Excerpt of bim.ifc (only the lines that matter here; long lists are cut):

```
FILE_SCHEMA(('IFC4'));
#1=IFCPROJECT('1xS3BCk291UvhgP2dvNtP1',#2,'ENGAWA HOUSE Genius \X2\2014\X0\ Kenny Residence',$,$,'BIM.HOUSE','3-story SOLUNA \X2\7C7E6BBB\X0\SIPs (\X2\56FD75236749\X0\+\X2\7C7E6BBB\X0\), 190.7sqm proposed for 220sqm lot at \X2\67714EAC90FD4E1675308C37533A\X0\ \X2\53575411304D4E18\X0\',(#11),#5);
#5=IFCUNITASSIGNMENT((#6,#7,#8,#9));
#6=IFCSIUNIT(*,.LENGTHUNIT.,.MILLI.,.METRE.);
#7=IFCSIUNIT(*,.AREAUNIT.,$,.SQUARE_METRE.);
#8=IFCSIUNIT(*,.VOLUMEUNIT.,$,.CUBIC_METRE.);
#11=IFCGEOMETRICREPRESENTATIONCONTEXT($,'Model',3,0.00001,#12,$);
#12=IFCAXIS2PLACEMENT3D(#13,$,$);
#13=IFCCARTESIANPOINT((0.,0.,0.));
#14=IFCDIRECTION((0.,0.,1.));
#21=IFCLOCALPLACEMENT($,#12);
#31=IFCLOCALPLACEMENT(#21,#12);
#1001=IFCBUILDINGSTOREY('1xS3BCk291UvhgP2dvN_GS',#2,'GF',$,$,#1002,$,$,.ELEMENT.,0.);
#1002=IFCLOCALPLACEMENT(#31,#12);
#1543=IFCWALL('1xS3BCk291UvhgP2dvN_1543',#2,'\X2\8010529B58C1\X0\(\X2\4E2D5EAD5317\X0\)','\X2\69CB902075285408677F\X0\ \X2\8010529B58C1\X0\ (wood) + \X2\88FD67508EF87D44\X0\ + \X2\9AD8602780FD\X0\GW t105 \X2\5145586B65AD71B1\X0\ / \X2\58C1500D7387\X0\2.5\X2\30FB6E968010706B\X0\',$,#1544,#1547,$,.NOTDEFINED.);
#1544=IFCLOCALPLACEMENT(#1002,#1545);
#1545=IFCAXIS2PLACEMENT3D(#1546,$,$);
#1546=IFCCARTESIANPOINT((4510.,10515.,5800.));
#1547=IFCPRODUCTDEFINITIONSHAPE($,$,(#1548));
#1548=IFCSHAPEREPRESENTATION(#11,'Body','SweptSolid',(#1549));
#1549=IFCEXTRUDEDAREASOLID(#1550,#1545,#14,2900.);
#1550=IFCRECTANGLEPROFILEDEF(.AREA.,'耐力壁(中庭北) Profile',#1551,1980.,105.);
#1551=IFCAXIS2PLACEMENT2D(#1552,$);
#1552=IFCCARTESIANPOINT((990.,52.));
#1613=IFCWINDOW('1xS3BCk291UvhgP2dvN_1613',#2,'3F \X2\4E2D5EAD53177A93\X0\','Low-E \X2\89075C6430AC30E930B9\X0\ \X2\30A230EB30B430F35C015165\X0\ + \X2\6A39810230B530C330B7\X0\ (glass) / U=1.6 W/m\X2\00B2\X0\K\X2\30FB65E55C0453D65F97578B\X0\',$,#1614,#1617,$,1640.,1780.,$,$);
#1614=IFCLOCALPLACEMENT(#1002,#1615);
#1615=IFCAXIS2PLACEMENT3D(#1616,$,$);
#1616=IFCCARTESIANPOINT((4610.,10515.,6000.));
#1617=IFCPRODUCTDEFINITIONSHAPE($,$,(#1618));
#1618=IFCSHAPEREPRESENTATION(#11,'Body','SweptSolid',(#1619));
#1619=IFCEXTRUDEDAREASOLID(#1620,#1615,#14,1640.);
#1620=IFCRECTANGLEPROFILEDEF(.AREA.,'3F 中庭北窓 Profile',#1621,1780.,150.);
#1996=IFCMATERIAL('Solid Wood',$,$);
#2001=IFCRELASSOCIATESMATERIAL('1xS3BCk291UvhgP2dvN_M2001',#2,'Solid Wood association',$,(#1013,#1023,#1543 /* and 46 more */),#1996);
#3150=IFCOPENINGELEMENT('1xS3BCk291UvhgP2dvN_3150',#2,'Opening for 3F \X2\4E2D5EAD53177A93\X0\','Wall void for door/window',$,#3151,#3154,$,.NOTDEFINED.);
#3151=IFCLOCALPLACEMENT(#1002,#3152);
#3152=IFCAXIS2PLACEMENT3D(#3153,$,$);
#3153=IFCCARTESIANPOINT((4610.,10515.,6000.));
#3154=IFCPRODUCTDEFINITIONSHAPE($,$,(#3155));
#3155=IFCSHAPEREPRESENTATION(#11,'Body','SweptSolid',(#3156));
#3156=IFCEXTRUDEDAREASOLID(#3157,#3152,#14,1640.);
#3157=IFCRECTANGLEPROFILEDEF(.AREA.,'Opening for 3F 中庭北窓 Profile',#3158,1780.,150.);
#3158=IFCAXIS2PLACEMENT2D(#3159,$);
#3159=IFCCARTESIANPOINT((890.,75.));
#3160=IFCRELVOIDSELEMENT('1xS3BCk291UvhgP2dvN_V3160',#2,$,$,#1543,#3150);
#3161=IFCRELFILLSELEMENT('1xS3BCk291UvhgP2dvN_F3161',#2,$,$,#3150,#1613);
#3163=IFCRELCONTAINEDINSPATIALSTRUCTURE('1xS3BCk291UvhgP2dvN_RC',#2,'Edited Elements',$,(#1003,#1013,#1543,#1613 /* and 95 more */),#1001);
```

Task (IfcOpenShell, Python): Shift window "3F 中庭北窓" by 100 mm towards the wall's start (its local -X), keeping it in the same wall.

```python
import ifcopenshell
import ifcopenshell.api.geometry
import ifcopenshell.util.placement

model = ifcopenshell.open("bim.ifc")

window = model.by_guid("1xS3BCk291UvhgP2dvN_1613")
opening = window.FillsVoids[0].RelatingOpeningElement
wall = opening.VoidsElements[0].RelatingBuildingElement

wall_matrix = ifcopenshell.util.placement.get_local_placement(wall.ObjectPlacement)
shift = wall_matrix[:3, 0] * -100.0
before = ifcopenshell.util.placement.get_local_placement(window.ObjectPlacement)[:3, 3].copy()

# The window is not placed relative to its opening, so move both.
for product in (opening, window):
    matrix = ifcopenshell.util.placement.get_local_placement(product.ObjectPlacement)
    matrix[:3, 3] += shift
    ifcopenshell.api.geometry.edit_object_placement(model, product=product, matrix=matrix, is_si=False)

after = ifcopenshell.util.placement.get_local_placement(window.ObjectPlacement)[:3, 3]
print("window moved by", (after - before).round(3) + 0.0)

model.write("bim_edited.ifc")
```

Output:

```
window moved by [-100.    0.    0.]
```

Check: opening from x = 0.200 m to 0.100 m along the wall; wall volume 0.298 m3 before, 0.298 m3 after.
